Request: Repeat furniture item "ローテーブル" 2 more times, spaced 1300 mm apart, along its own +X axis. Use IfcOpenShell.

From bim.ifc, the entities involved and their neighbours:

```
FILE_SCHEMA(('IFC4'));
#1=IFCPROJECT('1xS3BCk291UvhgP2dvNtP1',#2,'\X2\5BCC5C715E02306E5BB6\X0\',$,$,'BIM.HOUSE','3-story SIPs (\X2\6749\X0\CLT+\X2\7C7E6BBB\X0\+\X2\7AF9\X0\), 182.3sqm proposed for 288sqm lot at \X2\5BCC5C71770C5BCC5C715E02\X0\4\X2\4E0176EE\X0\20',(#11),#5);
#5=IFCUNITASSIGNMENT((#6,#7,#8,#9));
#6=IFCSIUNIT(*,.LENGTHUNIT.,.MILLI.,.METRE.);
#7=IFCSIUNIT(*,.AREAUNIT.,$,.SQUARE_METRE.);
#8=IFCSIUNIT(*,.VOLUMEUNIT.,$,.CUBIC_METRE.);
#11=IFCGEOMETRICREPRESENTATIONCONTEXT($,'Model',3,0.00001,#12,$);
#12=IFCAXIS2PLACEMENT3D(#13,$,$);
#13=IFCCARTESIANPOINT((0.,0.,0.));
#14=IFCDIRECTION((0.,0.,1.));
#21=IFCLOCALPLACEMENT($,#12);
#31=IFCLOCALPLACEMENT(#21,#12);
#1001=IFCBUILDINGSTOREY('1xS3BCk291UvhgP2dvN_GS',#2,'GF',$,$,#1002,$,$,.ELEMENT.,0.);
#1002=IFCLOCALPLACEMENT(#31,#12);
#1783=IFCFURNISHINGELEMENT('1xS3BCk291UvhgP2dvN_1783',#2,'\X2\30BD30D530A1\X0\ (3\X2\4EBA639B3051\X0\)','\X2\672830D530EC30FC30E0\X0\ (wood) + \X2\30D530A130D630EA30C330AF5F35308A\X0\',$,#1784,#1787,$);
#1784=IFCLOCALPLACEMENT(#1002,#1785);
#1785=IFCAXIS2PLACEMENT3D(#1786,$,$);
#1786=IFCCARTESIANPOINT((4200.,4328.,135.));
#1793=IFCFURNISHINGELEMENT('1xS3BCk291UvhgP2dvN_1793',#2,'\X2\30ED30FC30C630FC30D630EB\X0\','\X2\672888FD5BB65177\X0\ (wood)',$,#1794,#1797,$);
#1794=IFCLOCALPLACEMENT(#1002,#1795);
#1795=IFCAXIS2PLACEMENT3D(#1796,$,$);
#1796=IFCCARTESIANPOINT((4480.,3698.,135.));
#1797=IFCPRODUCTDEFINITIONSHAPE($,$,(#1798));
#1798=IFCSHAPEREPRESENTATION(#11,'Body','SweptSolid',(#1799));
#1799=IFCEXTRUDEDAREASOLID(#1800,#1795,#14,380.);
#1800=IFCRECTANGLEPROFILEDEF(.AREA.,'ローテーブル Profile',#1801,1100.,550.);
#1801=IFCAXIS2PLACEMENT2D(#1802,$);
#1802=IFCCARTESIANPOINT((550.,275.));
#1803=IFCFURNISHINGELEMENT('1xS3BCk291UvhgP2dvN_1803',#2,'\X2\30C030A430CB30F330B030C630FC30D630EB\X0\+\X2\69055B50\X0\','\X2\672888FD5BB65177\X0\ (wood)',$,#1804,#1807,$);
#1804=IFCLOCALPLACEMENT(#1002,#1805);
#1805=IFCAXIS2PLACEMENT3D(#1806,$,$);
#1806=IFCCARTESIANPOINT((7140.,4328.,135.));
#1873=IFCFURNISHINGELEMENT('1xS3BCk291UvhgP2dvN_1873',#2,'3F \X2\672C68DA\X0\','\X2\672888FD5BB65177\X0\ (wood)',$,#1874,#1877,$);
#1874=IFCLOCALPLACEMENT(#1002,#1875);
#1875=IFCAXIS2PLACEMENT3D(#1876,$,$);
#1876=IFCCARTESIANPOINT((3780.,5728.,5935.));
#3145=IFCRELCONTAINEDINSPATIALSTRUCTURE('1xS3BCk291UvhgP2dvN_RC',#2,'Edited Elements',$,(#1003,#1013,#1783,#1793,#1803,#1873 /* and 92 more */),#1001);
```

```python
import ifcopenshell
import ifcopenshell.api.geometry
import ifcopenshell.api.root
import ifcopenshell.util.element
import ifcopenshell.util.placement
import ifcopenshell.util.unit

model = ifcopenshell.open("bim.ifc")
unit_scale = ifcopenshell.util.unit.calculate_unit_scale(model)


def reuse_history(source, copy):
    """copy_class also copies each property set's owner history, people and application; keep the originals."""
    for rel in copy.IsDefinedBy:
        if rel.is_a("IfcRelDefinesByProperties") and (history := rel.RelatingPropertyDefinition.OwnerHistory):
            rel.RelatingPropertyDefinition.OwnerHistory = source.OwnerHistory
            ifcopenshell.util.element.remove_deep2(model, history)


source = model.by_guid("1xS3BCk291UvhgP2dvN_1793")
base = ifcopenshell.util.placement.get_local_placement(source.ObjectPlacement)
step = base[:3, 0] * 1.3 / unit_scale

for i in range(1, 3):
    copy = ifcopenshell.api.root.copy_class(model, product=source)
    copy.Representation = ifcopenshell.util.element.copy_deep(
        model, source.Representation, exclude=["IfcGeometricRepresentationContext", "IfcRepresentationMap"]
    )
    reuse_history(source, copy)
    matrix = base.copy()
    matrix[:3, 3] += i * step
    print("added at", matrix[:3, 3].round(3) + 0.0)
    ifcopenshell.api.geometry.edit_object_placement(model, product=copy, matrix=matrix, is_si=False)

model.write("bim_rev.ifc")
```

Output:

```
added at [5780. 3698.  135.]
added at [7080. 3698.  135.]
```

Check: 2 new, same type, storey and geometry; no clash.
